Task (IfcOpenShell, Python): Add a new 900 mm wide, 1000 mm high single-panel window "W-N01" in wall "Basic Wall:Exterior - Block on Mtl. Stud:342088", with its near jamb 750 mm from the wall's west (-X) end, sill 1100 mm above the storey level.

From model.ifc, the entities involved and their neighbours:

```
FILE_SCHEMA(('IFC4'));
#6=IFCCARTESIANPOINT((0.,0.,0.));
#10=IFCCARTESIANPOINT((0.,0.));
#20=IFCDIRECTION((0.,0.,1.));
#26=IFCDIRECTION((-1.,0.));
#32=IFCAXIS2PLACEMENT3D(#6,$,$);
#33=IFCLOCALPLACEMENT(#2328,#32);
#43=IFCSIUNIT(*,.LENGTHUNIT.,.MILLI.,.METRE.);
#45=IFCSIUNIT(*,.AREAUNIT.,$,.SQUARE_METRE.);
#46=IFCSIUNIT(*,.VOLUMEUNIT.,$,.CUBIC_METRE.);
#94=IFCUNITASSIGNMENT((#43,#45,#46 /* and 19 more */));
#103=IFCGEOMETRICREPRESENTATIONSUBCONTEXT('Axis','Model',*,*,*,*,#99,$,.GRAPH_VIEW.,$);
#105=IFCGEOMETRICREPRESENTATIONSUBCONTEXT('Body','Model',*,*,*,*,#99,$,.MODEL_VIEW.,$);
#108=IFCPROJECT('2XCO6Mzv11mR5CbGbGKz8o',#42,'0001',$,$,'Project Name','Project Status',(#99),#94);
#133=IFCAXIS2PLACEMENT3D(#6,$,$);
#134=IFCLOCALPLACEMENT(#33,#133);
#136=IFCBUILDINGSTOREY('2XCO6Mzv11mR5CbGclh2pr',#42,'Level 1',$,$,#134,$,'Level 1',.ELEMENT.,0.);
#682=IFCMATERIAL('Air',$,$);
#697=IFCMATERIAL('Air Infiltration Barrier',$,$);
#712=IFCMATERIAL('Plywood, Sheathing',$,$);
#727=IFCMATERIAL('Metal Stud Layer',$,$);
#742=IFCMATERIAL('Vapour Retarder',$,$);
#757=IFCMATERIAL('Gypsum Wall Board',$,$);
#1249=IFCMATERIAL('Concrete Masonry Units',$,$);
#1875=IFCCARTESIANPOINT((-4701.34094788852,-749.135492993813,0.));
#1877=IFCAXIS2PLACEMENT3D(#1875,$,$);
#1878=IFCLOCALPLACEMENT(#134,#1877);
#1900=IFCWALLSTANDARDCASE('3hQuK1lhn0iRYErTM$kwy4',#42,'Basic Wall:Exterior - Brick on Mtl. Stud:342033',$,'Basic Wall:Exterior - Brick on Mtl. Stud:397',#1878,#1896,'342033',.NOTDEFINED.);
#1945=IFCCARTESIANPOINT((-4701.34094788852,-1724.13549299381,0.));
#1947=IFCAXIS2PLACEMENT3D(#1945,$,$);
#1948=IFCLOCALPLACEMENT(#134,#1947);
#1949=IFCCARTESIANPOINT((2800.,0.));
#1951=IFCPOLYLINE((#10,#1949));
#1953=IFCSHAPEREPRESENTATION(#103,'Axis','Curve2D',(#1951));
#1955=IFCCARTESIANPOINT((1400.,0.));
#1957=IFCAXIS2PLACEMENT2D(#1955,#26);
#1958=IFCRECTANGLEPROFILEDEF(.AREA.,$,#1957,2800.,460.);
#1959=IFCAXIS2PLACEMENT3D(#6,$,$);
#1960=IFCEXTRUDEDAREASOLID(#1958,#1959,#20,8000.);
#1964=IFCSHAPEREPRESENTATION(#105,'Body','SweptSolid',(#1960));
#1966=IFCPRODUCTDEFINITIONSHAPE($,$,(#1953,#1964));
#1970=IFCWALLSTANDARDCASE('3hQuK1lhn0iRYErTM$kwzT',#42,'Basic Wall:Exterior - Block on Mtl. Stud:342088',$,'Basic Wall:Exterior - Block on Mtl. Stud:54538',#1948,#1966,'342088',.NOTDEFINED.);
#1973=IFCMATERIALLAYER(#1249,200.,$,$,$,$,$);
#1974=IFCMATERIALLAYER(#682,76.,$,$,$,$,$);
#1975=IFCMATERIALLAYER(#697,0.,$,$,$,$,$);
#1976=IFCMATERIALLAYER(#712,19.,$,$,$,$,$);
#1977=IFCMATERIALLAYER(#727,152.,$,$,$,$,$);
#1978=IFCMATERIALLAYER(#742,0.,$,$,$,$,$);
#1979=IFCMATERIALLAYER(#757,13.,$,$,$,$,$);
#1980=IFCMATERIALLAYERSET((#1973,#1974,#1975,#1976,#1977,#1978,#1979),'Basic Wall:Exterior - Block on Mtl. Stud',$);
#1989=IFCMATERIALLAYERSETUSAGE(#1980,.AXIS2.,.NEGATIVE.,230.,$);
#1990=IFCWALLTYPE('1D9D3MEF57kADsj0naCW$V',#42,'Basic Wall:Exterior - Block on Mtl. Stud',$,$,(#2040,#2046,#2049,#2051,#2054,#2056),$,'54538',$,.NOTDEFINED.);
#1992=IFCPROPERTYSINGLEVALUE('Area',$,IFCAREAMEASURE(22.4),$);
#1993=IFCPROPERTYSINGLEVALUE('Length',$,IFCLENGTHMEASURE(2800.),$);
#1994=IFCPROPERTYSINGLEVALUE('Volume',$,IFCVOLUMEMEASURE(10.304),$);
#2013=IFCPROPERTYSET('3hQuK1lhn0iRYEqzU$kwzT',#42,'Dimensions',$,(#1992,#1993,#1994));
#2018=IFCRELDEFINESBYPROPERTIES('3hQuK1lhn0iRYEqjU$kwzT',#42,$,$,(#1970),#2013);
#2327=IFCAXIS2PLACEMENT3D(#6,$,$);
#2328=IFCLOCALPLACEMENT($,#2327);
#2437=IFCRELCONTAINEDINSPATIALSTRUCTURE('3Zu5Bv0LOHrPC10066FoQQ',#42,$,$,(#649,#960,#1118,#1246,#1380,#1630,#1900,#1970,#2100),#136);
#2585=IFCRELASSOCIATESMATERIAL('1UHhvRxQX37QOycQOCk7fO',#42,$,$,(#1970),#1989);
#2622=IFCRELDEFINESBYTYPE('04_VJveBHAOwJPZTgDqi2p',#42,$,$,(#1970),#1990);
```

```python
import numpy as np
import ifcopenshell
import ifcopenshell.api.feature
import ifcopenshell.api.geometry
import ifcopenshell.api.pset
import ifcopenshell.api.root
import ifcopenshell.api.spatial
import ifcopenshell.geom
import ifcopenshell.util.element
import ifcopenshell.util.placement
import ifcopenshell.util.representation
import ifcopenshell.util.shape
import ifcopenshell.util.unit

model = ifcopenshell.open("model.ifc")
unit_scale = ifcopenshell.util.unit.calculate_unit_scale(model)
area_scale = ifcopenshell.util.unit.calculate_unit_scale(model, "AREAUNIT")
volume_scale = ifcopenshell.util.unit.calculate_unit_scale(model, "VOLUMEUNIT")
settings = ifcopenshell.geom.settings()


def volume(element):
    """Net volume in cubic metres, openings subtracted."""
    shape = ifcopenshell.geom.create_shape(settings, element)
    return ifcopenshell.util.shape.get_volume(shape.geometry)


wall = model.by_guid("3hQuK1lhn0iRYErTM$kwzT")
storey = ifcopenshell.util.element.get_container(wall, ifc_class="IfcBuildingStorey")
context = ifcopenshell.util.representation.get_context(model, "Model", "Body", "MODEL_VIEW")
before = volume(wall)

width, height, from_end, sill = 0.9, 1, 0.75, 1.1  # metres

# The wall runs along its own X axis, and the end named is its -X end.
wall_shape = ifcopenshell.geom.create_shape(settings, wall)
x, y, z = ifcopenshell.util.shape.get_vertices(wall_shape.geometry).T
start = x.min() + from_end
face, thickness = float(y.min()), float(y.max() - y.min())
wall_matrix = ifcopenshell.util.placement.get_local_placement(wall.ObjectPlacement)
level = ifcopenshell.util.placement.get_local_placement(storey.ObjectPlacement)[2, 3]


def in_wall(x, y):
    """Placement at x, y metres in the wall's axes, at sill height."""
    matrix = wall_matrix.copy()
    matrix[:, 3] = wall_matrix @ np.array([x / unit_scale, y / unit_scale, 0.0, 1.0])
    matrix[2, 3] = level + sill / unit_scale
    return matrix


# Opening: a box that overshoots both wall faces by 50 mm.
opening = ifcopenshell.api.root.create_entity(model, ifc_class="IfcOpeningElement", predefined_type="OPENING")
box = ifcopenshell.api.geometry.add_wall_representation(
    model, context=context, length=width, height=height, thickness=thickness + 0.1
)
ifcopenshell.api.geometry.assign_representation(model, product=opening, representation=box)
ifcopenshell.api.geometry.edit_object_placement(model, product=opening, matrix=in_wall(start, face - 0.05), is_si=False)
ifcopenshell.api.feature.add_feature(model, feature=opening, element=wall)

window = ifcopenshell.api.root.create_entity(model, ifc_class="IfcWindow", name="W-N01", predefined_type="WINDOW")
window.OverallWidth, window.OverallHeight = width / unit_scale, height / unit_scale
window.PartitioningType = "SINGLE_PANEL"
body = ifcopenshell.api.geometry.add_window_representation(
    model,
    context=context,
    overall_width=window.OverallWidth,
    overall_height=window.OverallHeight,
    partition_type="SINGLE_PANEL",
)
ifcopenshell.api.geometry.assign_representation(model, product=window, representation=body)
ifcopenshell.api.spatial.assign_container(model, products=[window], relating_structure=storey)
ifcopenshell.api.feature.add_filling(model, opening=opening, element=window)

# Centre the window in the wall's thickness.
ifcopenshell.api.geometry.edit_object_placement(model, product=window, matrix=in_wall(start, face), is_si=False)
window_shape = ifcopenshell.geom.create_shape(settings, window)
depth = ifcopenshell.util.shape.get_vertices(window_shape.geometry)[:, 1]
offset = face + thickness / 2 - (depth.min() + depth.max()) / 2
ifcopenshell.api.geometry.edit_object_placement(model, product=window, matrix=in_wall(start, offset), is_si=False)

after = volume(wall)

# Update the wall's stored quantities.
pset = model.by_id(ifcopenshell.util.element.get_pset(wall, "Dimensions", should_inherit=False)["id"])
ifcopenshell.api.pset.edit_pset(model, pset=pset, properties={
    "Area": model.create_entity("IfcAreaMeasure", after / thickness / area_scale),
    "Volume": model.create_entity("IfcVolumeMeasure", after / volume_scale),
})

print(f"wall volume {before:.3f} -> {after:.3f} m3")

model.write("model_edited.ifc")
```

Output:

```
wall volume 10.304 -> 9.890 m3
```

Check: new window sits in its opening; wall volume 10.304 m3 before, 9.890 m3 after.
